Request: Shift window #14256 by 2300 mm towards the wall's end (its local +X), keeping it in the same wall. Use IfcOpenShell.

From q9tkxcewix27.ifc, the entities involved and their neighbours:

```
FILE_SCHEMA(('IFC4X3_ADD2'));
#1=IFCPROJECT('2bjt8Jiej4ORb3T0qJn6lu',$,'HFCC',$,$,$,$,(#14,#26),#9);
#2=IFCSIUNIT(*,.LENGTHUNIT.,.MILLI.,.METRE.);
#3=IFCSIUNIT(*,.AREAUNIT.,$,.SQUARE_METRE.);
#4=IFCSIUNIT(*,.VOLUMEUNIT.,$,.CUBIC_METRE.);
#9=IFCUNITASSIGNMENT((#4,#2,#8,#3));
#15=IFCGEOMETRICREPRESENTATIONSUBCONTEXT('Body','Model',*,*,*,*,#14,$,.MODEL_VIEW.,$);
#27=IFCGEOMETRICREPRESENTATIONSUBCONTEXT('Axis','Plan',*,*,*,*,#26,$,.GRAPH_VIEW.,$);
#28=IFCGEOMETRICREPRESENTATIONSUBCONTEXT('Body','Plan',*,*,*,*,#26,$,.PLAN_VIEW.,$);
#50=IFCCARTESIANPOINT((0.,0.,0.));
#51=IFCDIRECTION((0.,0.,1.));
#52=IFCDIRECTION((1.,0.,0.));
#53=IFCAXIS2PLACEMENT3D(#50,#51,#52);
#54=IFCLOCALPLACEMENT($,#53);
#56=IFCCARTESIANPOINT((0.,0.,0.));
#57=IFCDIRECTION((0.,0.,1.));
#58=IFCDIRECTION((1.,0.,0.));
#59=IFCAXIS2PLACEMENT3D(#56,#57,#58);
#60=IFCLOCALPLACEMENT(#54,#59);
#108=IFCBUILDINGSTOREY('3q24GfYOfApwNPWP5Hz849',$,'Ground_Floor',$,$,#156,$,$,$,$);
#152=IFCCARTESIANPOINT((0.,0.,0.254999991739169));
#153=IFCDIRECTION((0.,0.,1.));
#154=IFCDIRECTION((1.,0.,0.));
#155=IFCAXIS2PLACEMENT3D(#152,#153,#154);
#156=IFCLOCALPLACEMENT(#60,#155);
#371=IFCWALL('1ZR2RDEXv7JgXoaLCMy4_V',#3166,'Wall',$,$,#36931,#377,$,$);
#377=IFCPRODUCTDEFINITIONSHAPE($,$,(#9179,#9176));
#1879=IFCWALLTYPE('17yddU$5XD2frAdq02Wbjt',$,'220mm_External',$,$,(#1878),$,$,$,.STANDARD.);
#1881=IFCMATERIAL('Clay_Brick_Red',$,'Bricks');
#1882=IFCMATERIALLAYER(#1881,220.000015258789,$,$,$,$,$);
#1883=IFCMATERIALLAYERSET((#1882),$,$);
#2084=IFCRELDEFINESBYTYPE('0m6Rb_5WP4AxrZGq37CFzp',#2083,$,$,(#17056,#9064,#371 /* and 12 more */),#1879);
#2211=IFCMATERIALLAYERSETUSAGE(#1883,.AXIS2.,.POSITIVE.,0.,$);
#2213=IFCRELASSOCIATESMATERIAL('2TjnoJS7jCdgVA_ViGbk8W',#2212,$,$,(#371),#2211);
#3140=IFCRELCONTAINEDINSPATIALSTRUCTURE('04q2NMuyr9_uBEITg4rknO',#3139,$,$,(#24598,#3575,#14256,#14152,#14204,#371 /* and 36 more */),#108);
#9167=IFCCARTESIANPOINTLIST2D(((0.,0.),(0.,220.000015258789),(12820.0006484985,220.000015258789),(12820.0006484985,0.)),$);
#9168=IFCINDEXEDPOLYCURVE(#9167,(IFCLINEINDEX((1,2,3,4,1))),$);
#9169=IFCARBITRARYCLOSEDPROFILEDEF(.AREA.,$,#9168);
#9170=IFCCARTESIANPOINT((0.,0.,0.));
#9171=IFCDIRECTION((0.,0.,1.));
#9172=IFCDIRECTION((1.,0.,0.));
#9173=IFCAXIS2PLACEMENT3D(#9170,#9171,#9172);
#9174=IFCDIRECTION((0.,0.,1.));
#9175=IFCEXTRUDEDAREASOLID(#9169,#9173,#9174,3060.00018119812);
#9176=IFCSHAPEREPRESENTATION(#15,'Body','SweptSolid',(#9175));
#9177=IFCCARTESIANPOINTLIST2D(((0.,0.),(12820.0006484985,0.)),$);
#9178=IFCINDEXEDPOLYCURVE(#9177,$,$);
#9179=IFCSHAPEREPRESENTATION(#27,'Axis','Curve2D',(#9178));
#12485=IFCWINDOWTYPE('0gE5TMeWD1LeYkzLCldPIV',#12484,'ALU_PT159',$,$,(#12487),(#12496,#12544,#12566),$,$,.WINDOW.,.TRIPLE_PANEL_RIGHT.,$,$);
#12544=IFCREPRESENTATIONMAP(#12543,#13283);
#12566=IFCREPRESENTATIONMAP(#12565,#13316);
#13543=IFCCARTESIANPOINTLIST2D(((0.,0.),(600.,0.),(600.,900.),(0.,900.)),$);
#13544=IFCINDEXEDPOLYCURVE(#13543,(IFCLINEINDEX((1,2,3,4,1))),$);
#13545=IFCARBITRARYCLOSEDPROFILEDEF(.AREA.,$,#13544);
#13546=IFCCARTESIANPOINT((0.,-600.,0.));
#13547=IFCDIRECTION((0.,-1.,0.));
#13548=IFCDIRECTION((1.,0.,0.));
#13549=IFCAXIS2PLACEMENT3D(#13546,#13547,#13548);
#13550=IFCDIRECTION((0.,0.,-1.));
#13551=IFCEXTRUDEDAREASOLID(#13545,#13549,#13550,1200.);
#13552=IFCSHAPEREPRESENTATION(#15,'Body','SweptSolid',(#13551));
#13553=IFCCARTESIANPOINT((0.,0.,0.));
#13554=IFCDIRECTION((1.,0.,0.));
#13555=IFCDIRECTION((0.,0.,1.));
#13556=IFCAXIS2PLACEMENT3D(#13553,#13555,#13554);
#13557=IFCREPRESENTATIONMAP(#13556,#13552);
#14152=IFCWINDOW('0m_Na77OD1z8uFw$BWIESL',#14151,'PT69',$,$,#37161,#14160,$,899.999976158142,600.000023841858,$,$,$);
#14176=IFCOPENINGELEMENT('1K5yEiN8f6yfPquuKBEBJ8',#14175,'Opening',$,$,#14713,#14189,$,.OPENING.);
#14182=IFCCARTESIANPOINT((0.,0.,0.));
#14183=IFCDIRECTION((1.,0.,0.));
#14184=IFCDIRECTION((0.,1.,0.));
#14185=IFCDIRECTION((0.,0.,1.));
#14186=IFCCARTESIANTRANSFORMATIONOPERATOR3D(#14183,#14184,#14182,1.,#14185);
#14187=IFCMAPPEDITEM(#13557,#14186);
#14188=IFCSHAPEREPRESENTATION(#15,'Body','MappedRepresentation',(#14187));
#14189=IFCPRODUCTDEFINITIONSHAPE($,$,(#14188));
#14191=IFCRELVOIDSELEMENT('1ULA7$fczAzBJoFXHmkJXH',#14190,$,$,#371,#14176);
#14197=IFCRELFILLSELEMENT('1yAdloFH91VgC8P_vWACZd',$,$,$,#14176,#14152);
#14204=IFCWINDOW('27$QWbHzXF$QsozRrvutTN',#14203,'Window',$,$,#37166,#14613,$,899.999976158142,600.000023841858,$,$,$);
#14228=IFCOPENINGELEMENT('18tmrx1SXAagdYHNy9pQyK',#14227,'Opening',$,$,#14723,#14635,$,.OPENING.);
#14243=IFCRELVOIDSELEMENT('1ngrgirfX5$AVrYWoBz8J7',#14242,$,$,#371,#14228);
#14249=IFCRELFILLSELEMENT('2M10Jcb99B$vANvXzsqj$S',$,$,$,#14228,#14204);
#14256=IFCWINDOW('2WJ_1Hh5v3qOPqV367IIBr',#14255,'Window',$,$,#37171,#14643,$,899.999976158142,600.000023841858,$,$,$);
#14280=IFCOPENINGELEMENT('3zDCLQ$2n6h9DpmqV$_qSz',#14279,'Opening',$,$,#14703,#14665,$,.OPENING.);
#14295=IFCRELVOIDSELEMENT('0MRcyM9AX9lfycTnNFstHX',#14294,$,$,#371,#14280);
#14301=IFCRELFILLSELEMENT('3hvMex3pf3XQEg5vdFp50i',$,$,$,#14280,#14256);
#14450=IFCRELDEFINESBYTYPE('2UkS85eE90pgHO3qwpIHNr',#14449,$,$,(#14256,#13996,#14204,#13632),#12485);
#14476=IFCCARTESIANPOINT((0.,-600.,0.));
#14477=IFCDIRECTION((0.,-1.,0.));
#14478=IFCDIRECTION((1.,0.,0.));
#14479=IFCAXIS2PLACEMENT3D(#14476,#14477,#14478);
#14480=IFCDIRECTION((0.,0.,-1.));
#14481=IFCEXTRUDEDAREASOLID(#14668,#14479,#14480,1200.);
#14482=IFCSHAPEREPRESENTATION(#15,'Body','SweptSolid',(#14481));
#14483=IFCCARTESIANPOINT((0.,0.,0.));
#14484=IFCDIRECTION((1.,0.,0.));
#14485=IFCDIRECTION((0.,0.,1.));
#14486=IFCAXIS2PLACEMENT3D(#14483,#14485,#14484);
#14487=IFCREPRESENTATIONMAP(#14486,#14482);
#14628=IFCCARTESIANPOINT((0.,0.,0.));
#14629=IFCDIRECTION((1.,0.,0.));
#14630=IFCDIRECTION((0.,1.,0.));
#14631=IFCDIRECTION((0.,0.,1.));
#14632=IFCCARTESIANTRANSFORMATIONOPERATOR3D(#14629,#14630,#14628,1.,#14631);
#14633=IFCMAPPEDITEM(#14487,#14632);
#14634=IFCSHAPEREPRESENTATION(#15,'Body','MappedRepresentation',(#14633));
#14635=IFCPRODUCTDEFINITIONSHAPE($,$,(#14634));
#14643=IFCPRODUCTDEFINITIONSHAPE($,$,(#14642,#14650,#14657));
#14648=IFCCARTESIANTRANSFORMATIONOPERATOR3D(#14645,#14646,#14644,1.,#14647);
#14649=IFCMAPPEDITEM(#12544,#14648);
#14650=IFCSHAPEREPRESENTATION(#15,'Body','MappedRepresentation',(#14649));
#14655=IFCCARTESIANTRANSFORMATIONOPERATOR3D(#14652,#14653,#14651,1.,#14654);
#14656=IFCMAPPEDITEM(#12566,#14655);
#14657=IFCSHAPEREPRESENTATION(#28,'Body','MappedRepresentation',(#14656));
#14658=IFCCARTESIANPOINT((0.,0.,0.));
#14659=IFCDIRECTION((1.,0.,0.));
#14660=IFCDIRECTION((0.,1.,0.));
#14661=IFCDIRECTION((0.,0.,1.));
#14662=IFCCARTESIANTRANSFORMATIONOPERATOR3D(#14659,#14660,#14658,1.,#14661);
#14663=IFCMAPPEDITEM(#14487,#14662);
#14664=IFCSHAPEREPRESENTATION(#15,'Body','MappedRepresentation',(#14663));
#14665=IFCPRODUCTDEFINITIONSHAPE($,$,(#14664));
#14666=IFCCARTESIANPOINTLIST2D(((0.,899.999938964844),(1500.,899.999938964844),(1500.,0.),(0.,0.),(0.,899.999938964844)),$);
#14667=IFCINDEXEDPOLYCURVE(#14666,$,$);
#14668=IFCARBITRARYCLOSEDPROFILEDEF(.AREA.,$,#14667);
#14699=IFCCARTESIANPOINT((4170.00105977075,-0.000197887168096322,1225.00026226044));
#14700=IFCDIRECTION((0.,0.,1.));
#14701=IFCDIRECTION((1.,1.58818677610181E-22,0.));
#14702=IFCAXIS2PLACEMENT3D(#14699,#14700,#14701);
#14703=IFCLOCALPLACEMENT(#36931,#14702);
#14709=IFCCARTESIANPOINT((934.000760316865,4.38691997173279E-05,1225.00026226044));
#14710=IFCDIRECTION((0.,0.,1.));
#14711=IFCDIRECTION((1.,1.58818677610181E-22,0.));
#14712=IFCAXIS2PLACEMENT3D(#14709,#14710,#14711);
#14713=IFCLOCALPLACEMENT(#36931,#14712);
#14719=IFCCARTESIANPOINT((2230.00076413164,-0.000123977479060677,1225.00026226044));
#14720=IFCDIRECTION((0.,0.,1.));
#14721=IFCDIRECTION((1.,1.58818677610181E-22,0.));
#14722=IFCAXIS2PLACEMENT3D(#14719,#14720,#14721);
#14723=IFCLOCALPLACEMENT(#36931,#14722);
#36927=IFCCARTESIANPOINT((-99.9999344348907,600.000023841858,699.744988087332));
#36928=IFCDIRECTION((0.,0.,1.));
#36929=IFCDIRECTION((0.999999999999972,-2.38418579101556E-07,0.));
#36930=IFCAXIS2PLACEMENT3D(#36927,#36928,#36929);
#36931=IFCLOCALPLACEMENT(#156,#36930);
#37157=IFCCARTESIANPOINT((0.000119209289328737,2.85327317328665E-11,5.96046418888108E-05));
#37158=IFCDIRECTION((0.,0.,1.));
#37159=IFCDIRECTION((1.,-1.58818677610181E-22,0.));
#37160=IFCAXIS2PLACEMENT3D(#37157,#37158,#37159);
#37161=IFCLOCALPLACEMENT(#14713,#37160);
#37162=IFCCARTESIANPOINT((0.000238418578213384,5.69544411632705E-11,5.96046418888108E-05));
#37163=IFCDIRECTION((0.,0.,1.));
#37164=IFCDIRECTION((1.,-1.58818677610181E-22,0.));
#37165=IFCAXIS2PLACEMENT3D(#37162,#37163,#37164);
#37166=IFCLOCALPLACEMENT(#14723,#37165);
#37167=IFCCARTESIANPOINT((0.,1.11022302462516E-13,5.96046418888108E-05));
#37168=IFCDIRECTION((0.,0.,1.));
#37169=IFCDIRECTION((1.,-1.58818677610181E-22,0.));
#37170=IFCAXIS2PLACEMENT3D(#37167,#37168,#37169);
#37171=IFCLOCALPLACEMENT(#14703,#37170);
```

```python
import ifcopenshell
import ifcopenshell.api.geometry
import ifcopenshell.util.placement
import ifcopenshell.util.unit

model = ifcopenshell.open("q9tkxcewix27.ifc")
unit_scale = ifcopenshell.util.unit.calculate_unit_scale(model)

window = model.by_id(14256)
opening = window.FillsVoids[0].RelatingOpeningElement
wall = opening.VoidsElements[0].RelatingBuildingElement

wall_matrix = ifcopenshell.util.placement.get_local_placement(wall.ObjectPlacement)
shift = wall_matrix[:3, 0] * 2.3 / unit_scale
before = ifcopenshell.util.placement.get_local_placement(window.ObjectPlacement)[:3, 3].copy()

# The window is placed relative to its opening, so it follows when the opening moves.
matrix = ifcopenshell.util.placement.get_local_placement(opening.ObjectPlacement)
matrix[:3, 3] += shift
ifcopenshell.api.geometry.edit_object_placement(
    model, product=opening, matrix=matrix, is_si=False, should_transform_children=True
)

after = ifcopenshell.util.placement.get_local_placement(window.ObjectPlacement)[:3, 3]
print("window moved by", (after - before).round(3) + 0.0)

model.write("q9tkxcewix27_rev.ifc")
```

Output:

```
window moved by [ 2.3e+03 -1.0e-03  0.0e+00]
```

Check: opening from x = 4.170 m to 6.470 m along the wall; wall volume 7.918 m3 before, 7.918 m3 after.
